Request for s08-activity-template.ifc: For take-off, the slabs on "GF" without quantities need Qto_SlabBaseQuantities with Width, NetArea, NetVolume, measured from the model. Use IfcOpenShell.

First a look at what the model holds.

```python
import ifcopenshell
import ifcopenshell.util.element
import ifcopenshell.util.unit

model = ifcopenshell.open("s08-activity-template.ifc")
print(model.schema)
for unit_type in ("LENGTHUNIT", "AREAUNIT", "VOLUMEUNIT"):
    print(unit_type, ifcopenshell.util.unit.calculate_unit_scale(model, unit_type))
storey = next(s for s in model.by_type("IfcBuildingStorey") if s.Name == "GF")
slabs = [e for e in ifcopenshell.util.element.get_decomposition(storey) if e.is_a("IfcSlab")]
for e in sorted(slabs, key=lambda e: e.id()):
    print(e.id(), e.is_a(), e.Name, list(ifcopenshell.util.element.get_psets(e, qtos_only=True)), sep=" | ")
```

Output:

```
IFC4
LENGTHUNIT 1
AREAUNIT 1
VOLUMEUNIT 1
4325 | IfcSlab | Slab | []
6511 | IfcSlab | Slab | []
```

```python
import ifcopenshell
import ifcopenshell.api.pset
import ifcopenshell.geom
import ifcopenshell.util.element
import ifcopenshell.util.shape
import ifcopenshell.util.unit

model = ifcopenshell.open("s08-activity-template.ifc")
unit_scale = ifcopenshell.util.unit.calculate_unit_scale(model)
area_scale = ifcopenshell.util.unit.calculate_unit_scale(model, "AREAUNIT")
volume_scale = ifcopenshell.util.unit.calculate_unit_scale(model, "VOLUMEUNIT")
settings = ifcopenshell.geom.settings()

storey = next(s for s in model.by_type("IfcBuildingStorey") if s.Name == "GF")
slabs = [e for e in ifcopenshell.util.element.get_decomposition(storey) if e.is_a("IfcSlab")]

for e in sorted(slabs, key=lambda e: e.id()):
    if ifcopenshell.util.element.get_psets(e, qtos_only=True, should_inherit=False):
        continue
    # Geometry comes back in metres, in the element's own axes.
    shape = ifcopenshell.geom.create_shape(settings, e)
    values = {
        "Width": ifcopenshell.util.shape.get_z(shape.geometry) / unit_scale,
        "NetArea": ifcopenshell.util.shape.get_footprint_area(shape.geometry) / area_scale,
        "NetVolume": ifcopenshell.util.shape.get_volume(shape.geometry) / volume_scale,
    }
    qto = ifcopenshell.api.pset.add_qto(model, product=e, name="Qto_SlabBaseQuantities")
    ifcopenshell.api.pset.edit_qto(model, qto=qto, properties=values)
    print(e.id(), {k: round(v, 3) for k, v in values.items()})

model.write("s08-activity-template_v2.ifc")
```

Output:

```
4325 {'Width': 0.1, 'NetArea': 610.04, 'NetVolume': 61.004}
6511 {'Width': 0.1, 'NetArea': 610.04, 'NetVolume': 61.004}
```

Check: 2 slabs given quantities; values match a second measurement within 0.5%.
